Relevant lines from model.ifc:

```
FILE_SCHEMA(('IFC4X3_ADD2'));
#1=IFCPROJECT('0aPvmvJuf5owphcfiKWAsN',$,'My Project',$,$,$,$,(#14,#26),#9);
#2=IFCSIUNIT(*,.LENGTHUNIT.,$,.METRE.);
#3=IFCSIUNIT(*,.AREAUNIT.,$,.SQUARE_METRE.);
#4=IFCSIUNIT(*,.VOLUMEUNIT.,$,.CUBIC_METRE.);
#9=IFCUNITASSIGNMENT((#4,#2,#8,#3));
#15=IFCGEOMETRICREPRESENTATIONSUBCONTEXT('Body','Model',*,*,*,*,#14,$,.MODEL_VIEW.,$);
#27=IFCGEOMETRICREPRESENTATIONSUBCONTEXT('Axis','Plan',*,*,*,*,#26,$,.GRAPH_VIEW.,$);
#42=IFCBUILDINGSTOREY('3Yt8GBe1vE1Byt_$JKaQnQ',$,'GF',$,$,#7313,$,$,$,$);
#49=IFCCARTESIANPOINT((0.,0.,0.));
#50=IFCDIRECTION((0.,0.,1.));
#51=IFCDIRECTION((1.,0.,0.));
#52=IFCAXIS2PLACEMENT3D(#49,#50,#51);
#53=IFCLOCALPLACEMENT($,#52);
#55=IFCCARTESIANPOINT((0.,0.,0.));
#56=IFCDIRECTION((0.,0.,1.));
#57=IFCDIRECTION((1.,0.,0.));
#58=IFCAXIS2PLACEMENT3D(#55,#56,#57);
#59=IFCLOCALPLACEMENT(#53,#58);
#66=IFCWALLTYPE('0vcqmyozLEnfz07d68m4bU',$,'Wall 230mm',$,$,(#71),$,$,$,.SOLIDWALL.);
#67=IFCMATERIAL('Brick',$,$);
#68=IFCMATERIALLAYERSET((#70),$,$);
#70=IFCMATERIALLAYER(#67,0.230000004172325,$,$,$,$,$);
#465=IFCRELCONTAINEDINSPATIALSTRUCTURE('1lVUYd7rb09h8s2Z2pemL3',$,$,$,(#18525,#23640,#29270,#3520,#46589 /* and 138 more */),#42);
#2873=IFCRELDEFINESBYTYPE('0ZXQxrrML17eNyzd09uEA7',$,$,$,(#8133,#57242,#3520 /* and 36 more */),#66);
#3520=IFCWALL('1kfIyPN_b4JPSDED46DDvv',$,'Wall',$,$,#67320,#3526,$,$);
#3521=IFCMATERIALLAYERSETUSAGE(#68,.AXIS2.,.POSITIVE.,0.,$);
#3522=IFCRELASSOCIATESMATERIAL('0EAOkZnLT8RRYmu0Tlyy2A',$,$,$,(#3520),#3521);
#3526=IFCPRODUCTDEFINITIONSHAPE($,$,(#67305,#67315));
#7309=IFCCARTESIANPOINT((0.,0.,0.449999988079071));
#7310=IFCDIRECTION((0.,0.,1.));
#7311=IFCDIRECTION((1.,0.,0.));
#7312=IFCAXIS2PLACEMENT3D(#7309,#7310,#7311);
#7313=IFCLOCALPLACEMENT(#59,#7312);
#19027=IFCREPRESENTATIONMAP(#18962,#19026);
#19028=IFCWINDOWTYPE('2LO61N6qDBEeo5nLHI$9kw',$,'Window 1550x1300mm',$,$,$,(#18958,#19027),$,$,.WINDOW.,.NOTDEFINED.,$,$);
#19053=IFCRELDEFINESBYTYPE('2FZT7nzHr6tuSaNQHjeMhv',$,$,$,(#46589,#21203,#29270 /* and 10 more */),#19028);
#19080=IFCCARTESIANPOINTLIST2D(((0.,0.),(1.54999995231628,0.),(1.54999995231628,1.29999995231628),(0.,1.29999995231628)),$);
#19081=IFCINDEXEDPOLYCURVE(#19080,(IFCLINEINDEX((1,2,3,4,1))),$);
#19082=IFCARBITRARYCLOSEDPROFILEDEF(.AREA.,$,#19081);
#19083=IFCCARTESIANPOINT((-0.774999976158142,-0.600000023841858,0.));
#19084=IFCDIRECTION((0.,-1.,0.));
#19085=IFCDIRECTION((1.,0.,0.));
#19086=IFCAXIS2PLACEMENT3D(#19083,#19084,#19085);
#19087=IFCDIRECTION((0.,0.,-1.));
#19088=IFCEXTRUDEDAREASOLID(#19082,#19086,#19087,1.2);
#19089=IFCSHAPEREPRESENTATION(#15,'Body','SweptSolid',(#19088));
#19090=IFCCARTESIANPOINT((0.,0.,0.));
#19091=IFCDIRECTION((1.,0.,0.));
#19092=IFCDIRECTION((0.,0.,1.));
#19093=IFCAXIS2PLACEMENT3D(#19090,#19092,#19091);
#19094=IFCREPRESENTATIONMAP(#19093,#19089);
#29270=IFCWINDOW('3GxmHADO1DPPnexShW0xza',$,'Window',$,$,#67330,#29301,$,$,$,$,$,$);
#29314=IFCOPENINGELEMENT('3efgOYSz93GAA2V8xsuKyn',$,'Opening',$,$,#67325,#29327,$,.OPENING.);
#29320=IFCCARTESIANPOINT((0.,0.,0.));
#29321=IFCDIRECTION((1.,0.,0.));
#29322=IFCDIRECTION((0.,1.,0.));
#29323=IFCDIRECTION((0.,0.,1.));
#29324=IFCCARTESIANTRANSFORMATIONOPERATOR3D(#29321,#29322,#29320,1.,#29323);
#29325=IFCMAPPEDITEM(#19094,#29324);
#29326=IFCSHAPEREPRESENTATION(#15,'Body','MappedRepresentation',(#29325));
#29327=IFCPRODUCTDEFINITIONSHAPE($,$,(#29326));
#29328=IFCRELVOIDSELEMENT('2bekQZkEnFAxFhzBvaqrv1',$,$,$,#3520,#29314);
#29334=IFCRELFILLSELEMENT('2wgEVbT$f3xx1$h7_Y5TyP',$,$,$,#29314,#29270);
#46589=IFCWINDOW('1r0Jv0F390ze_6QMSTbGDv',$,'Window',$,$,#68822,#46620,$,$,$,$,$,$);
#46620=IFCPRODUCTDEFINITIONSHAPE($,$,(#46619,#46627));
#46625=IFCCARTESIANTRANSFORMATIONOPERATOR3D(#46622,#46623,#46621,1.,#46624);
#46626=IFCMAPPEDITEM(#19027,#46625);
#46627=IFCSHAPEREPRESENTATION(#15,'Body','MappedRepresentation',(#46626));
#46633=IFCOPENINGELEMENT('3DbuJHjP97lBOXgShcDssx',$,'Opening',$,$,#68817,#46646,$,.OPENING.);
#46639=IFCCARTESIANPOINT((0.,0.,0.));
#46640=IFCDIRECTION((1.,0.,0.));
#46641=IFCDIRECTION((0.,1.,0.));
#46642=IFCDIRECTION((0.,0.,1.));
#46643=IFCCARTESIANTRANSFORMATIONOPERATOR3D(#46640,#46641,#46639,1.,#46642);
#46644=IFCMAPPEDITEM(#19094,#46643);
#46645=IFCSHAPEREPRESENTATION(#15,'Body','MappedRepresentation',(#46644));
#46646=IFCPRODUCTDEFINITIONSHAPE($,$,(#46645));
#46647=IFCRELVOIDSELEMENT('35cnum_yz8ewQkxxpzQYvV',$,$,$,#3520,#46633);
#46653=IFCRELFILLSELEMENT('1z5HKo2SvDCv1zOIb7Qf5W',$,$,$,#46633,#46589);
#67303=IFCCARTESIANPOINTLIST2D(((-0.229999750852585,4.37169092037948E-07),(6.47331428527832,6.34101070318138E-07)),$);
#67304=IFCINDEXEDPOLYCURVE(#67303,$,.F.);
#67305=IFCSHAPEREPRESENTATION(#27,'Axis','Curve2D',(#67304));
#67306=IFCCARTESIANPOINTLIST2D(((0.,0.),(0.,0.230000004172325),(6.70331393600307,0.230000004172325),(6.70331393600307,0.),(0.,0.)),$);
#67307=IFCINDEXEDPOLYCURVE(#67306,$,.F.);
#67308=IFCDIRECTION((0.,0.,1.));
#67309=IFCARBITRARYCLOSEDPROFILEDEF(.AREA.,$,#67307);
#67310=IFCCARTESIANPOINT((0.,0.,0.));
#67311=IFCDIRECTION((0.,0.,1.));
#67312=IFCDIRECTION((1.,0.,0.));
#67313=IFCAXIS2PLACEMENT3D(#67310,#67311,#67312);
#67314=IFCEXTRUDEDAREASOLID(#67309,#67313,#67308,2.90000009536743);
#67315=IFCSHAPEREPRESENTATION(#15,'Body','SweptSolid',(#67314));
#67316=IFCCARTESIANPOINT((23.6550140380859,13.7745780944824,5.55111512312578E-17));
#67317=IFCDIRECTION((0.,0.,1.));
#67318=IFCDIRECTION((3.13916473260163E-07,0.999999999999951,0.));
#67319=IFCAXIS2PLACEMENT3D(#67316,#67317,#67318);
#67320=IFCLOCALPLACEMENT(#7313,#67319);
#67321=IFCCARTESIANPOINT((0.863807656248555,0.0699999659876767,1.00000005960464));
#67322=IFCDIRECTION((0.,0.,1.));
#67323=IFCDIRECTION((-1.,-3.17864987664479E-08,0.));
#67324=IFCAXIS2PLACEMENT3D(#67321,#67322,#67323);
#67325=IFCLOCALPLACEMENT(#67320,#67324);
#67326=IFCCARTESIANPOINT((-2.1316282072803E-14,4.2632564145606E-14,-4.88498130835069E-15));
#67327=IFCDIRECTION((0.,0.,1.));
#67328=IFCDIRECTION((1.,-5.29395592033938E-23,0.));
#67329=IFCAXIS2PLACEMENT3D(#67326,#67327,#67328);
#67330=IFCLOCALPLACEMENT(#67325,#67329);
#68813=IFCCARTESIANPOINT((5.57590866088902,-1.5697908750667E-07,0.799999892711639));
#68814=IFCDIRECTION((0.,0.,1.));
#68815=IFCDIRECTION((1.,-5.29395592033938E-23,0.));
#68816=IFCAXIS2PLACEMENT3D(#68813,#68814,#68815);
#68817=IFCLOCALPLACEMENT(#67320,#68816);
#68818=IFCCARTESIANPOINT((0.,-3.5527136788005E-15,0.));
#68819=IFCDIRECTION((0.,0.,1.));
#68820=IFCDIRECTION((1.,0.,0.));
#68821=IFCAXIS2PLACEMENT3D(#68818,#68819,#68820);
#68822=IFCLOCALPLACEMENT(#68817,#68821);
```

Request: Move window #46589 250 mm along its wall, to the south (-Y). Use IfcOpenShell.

```python
import ifcopenshell
import ifcopenshell.api.geometry
import ifcopenshell.util.placement

model = ifcopenshell.open("model.ifc")

window = model.by_guid("1r0Jv0F390ze_6QMSTbGDv")
opening = window.FillsVoids[0].RelatingOpeningElement
wall = opening.VoidsElements[0].RelatingBuildingElement

wall_matrix = ifcopenshell.util.placement.get_local_placement(wall.ObjectPlacement)
shift = wall_matrix[:3, 0] * -0.25
before = ifcopenshell.util.placement.get_local_placement(window.ObjectPlacement)[:3, 3].copy()

# The window is placed relative to its opening, so it follows when the opening moves.
matrix = ifcopenshell.util.placement.get_local_placement(opening.ObjectPlacement)
matrix[:3, 3] += shift
ifcopenshell.api.geometry.edit_object_placement(
    model, product=opening, matrix=matrix, is_si=False, should_transform_children=True
)

after = ifcopenshell.util.placement.get_local_placement(window.ObjectPlacement)[:3, 3]
print("window moved by", (after - before).round(3) + 0.0)

model.write("model_edited.ifc")
```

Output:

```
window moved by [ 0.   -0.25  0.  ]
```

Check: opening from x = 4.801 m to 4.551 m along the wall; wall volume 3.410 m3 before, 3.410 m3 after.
